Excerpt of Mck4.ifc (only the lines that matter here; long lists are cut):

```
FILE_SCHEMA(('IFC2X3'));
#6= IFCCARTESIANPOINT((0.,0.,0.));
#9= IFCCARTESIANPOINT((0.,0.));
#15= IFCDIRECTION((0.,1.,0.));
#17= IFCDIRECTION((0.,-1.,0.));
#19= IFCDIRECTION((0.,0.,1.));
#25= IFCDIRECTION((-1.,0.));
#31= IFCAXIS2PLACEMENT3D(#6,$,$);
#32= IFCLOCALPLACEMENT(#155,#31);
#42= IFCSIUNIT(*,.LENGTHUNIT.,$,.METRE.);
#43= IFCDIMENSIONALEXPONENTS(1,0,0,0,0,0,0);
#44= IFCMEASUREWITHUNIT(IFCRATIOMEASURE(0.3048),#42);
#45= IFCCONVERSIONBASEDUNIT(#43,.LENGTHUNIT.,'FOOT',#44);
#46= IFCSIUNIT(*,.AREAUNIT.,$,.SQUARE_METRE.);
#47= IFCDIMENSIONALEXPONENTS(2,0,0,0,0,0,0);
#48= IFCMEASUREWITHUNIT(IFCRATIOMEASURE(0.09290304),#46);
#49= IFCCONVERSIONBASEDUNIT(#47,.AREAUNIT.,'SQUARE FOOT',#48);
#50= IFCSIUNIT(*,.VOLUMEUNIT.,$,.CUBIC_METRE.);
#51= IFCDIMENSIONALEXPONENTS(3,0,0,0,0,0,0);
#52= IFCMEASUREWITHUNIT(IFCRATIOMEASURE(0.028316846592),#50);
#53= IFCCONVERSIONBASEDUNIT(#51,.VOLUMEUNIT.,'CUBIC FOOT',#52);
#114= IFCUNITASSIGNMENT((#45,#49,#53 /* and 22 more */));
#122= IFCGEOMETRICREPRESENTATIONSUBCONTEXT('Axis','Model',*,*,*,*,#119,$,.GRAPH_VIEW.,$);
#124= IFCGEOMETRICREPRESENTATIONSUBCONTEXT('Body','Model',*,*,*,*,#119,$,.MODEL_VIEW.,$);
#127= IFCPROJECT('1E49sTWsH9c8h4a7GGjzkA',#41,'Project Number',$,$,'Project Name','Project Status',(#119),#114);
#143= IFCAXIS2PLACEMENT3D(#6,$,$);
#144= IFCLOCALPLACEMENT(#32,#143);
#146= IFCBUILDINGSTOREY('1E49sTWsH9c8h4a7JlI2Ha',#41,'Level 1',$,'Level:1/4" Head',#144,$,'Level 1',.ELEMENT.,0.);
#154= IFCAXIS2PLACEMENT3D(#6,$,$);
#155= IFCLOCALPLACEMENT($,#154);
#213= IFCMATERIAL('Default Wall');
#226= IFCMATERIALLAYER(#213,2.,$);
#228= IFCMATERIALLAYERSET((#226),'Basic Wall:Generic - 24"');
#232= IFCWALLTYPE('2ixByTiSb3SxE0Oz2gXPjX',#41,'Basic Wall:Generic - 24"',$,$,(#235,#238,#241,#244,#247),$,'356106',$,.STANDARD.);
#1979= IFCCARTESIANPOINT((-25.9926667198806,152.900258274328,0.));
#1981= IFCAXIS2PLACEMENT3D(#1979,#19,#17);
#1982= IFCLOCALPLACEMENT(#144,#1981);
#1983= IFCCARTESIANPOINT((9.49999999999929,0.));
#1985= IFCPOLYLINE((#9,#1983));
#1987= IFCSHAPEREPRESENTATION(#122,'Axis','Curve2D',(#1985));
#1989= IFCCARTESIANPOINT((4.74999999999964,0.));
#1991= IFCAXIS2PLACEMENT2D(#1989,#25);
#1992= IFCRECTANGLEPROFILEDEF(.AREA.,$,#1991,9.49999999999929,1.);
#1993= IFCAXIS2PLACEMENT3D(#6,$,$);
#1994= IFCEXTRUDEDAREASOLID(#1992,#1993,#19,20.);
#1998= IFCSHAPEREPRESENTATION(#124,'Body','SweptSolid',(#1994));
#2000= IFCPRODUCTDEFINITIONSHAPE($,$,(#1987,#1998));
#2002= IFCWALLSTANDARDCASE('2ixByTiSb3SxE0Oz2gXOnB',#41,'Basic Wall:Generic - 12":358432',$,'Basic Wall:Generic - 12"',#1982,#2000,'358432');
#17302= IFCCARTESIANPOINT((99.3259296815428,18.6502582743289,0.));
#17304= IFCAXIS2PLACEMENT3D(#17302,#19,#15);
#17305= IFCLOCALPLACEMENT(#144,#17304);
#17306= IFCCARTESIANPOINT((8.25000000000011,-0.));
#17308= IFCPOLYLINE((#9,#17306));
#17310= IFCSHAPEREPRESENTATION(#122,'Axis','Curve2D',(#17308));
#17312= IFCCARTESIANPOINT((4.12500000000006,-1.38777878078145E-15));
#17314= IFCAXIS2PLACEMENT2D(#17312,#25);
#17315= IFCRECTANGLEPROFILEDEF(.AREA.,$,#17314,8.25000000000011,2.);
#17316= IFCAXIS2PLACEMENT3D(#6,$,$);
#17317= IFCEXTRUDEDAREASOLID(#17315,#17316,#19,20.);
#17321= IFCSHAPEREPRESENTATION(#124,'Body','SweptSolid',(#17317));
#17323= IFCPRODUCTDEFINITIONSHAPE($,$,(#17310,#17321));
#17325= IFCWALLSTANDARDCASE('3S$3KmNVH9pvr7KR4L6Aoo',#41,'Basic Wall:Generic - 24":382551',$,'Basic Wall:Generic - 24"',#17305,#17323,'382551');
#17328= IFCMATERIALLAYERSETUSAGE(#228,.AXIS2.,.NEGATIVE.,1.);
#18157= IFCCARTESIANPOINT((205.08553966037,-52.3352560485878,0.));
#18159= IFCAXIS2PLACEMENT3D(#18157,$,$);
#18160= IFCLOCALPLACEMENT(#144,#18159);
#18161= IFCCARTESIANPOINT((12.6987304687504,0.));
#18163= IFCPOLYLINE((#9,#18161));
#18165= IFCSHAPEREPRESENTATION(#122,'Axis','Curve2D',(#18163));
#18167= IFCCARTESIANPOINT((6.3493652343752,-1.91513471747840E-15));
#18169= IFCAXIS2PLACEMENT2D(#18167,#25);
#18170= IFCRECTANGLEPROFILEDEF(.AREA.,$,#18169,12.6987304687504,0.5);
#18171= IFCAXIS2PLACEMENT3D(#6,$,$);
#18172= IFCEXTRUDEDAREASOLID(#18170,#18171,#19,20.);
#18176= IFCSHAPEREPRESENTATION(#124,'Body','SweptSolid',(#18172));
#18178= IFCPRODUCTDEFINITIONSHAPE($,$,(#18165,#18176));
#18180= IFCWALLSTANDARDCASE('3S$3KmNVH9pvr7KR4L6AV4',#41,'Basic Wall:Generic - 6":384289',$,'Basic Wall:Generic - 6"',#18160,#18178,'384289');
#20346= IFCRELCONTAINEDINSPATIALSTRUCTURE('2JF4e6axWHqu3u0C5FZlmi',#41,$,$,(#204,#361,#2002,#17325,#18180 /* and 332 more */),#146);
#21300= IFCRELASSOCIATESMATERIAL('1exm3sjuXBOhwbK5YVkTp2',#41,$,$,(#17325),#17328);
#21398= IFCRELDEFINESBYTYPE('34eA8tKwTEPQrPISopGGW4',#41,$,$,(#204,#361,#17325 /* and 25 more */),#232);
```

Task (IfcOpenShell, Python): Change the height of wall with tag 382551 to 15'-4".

```python
import ifcopenshell
import ifcopenshell.geom
import ifcopenshell.util.representation
import ifcopenshell.util.shape
import ifcopenshell.util.unit

model = ifcopenshell.open("Mck4.ifc")
unit_scale = ifcopenshell.util.unit.calculate_unit_scale(model)
settings = ifcopenshell.geom.settings()


def volume(element):
    """Net volume in cubic metres, openings subtracted."""
    shape = ifcopenshell.geom.create_shape(settings, element)
    return ifcopenshell.util.shape.get_volume(shape.geometry)


wall = model.by_guid("3S$3KmNVH9pvr7KR4L6Aoo")
before = volume(wall)

body = ifcopenshell.util.representation.get_representation(wall, "Model", "Body")
solid = body.Items[0]
old_height = solid.Depth
solid.Depth = 184 * 0.0254 / unit_scale
after = volume(wall)

print(f"height {old_height:g} -> {solid.Depth:g}, volume {before:.3f} -> {after:.3f} m3")

model.write("Mck4_edited.ifc")
```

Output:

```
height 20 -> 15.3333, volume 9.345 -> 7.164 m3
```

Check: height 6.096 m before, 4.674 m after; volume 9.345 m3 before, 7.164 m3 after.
